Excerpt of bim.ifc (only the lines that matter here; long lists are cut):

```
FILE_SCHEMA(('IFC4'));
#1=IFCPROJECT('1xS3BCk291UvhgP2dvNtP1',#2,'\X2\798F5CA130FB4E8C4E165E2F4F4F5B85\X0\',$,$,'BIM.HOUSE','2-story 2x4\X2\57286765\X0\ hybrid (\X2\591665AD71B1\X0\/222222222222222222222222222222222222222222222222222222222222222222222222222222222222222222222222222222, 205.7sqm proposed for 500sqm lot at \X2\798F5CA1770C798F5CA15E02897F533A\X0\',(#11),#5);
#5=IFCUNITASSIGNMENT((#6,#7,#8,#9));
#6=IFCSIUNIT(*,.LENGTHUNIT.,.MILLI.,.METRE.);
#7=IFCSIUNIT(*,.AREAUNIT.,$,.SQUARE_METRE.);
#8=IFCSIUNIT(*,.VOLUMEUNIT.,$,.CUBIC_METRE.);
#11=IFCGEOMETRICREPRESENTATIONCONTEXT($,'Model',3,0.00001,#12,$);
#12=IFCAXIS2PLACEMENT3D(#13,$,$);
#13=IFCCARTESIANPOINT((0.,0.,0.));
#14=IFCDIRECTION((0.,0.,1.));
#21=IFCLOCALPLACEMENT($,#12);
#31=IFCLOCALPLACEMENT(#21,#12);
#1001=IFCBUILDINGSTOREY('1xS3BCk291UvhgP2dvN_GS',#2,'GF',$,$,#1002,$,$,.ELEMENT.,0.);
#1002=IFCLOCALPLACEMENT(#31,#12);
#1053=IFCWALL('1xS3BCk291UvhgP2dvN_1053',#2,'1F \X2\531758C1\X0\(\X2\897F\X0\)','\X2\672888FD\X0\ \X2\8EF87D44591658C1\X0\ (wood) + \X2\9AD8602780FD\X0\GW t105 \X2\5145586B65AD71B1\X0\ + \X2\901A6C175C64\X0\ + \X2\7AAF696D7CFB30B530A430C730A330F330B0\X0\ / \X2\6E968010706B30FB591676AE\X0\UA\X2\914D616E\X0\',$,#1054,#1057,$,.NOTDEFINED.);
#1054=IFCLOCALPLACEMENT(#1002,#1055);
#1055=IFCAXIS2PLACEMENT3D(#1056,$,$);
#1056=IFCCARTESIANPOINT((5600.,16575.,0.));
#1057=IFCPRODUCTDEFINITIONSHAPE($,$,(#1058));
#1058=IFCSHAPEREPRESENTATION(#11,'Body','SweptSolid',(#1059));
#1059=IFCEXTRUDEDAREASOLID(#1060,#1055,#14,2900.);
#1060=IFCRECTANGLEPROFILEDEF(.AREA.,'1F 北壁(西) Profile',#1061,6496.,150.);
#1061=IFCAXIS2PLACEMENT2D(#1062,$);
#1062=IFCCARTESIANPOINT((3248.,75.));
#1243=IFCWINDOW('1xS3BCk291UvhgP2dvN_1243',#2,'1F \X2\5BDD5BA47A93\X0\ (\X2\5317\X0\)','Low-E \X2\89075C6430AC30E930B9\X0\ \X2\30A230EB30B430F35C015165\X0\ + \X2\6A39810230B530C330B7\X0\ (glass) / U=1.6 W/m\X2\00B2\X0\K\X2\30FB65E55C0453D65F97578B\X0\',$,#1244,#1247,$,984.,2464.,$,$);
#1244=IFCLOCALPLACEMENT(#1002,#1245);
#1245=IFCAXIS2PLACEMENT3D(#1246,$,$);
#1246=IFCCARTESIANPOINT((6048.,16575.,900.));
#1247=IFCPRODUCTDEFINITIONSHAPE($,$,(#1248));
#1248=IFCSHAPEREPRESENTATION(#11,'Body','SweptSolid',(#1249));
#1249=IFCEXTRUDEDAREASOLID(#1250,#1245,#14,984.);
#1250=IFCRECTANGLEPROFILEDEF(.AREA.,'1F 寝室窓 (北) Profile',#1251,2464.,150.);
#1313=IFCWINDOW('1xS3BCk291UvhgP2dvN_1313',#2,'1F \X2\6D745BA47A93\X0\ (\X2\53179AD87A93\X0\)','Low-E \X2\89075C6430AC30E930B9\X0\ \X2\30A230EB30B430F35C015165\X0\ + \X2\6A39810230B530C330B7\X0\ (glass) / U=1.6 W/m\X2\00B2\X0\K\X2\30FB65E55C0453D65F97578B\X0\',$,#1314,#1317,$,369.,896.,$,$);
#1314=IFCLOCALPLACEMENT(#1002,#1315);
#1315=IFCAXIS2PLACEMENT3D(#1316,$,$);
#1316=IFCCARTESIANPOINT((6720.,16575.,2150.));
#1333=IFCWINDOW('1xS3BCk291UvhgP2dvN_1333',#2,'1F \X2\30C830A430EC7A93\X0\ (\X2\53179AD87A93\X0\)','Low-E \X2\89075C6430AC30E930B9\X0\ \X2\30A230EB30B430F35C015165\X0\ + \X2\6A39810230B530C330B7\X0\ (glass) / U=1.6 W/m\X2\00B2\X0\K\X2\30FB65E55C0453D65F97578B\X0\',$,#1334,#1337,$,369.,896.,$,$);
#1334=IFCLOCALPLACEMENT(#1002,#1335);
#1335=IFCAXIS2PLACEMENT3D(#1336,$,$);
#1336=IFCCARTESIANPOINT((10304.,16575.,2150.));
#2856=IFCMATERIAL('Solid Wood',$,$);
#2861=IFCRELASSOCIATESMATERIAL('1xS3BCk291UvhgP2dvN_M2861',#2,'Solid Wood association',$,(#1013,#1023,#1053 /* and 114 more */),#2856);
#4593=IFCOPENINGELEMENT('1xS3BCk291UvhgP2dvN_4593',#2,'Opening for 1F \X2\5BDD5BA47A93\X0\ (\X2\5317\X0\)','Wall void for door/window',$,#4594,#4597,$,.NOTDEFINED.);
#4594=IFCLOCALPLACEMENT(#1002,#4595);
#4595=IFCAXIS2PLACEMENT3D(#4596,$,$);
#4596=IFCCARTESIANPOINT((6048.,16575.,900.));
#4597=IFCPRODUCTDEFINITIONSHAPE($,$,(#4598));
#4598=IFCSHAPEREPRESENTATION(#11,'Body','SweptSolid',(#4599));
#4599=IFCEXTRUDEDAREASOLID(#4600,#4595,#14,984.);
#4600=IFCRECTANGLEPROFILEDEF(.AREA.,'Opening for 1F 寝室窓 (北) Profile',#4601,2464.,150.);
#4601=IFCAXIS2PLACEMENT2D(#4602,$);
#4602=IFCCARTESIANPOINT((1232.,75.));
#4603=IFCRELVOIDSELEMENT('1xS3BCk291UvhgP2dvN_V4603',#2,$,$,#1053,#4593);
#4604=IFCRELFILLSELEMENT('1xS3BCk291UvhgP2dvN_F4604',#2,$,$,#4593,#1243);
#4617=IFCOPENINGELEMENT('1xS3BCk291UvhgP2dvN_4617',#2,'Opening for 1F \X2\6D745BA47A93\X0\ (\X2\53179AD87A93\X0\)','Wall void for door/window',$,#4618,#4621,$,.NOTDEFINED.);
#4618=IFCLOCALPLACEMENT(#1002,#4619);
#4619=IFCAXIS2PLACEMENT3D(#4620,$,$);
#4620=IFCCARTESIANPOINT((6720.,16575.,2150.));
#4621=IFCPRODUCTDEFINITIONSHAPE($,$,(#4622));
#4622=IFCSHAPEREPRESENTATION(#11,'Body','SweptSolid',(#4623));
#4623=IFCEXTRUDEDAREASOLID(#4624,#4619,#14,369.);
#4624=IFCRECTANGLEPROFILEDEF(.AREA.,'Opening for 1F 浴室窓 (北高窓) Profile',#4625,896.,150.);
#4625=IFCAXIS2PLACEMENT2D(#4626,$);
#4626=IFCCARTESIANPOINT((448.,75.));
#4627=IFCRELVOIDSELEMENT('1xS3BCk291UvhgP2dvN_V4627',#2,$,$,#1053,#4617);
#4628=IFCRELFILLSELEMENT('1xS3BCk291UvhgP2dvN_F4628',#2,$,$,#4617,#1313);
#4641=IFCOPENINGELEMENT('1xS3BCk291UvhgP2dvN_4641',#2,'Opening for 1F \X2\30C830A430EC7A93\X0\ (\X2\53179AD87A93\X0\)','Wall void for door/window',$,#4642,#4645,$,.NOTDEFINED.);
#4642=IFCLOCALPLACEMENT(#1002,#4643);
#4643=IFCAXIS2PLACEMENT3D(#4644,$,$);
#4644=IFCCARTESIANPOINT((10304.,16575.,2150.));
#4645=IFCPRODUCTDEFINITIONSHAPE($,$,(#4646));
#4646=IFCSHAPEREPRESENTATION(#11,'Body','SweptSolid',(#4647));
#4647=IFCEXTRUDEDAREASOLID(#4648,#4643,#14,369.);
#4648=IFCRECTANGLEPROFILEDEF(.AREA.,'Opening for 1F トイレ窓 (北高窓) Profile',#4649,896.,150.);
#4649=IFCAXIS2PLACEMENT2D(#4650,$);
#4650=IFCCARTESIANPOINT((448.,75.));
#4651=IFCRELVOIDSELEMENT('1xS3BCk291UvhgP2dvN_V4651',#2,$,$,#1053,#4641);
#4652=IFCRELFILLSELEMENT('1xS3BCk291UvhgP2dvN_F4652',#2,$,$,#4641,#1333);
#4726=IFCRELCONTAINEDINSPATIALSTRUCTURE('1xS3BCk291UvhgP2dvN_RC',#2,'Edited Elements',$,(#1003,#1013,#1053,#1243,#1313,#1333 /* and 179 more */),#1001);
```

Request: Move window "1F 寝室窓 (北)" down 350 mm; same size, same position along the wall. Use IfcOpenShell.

```python
import numpy as np
import ifcopenshell
import ifcopenshell.api.geometry
import ifcopenshell.util.placement
import ifcopenshell.util.unit

model = ifcopenshell.open("bim.ifc")
unit_scale = ifcopenshell.util.unit.calculate_unit_scale(model)

window = model.by_guid("1xS3BCk291UvhgP2dvN_1243")
opening = window.FillsVoids[0].RelatingOpeningElement
dz = -0.35 / unit_scale

shift = np.array([0.0, 0.0, dz])
# The window is not placed relative to its opening, so move both.
for product in (opening, window):
    matrix = ifcopenshell.util.placement.get_local_placement(product.ObjectPlacement)
    matrix[:3, 3] += shift
    ifcopenshell.api.geometry.edit_object_placement(model, product=product, matrix=matrix, is_si=False)

print(f"moved by {dz * unit_scale:+.3f} m")

model.write("bim_edited.ifc")
```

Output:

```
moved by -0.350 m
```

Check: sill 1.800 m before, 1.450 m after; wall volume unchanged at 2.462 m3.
